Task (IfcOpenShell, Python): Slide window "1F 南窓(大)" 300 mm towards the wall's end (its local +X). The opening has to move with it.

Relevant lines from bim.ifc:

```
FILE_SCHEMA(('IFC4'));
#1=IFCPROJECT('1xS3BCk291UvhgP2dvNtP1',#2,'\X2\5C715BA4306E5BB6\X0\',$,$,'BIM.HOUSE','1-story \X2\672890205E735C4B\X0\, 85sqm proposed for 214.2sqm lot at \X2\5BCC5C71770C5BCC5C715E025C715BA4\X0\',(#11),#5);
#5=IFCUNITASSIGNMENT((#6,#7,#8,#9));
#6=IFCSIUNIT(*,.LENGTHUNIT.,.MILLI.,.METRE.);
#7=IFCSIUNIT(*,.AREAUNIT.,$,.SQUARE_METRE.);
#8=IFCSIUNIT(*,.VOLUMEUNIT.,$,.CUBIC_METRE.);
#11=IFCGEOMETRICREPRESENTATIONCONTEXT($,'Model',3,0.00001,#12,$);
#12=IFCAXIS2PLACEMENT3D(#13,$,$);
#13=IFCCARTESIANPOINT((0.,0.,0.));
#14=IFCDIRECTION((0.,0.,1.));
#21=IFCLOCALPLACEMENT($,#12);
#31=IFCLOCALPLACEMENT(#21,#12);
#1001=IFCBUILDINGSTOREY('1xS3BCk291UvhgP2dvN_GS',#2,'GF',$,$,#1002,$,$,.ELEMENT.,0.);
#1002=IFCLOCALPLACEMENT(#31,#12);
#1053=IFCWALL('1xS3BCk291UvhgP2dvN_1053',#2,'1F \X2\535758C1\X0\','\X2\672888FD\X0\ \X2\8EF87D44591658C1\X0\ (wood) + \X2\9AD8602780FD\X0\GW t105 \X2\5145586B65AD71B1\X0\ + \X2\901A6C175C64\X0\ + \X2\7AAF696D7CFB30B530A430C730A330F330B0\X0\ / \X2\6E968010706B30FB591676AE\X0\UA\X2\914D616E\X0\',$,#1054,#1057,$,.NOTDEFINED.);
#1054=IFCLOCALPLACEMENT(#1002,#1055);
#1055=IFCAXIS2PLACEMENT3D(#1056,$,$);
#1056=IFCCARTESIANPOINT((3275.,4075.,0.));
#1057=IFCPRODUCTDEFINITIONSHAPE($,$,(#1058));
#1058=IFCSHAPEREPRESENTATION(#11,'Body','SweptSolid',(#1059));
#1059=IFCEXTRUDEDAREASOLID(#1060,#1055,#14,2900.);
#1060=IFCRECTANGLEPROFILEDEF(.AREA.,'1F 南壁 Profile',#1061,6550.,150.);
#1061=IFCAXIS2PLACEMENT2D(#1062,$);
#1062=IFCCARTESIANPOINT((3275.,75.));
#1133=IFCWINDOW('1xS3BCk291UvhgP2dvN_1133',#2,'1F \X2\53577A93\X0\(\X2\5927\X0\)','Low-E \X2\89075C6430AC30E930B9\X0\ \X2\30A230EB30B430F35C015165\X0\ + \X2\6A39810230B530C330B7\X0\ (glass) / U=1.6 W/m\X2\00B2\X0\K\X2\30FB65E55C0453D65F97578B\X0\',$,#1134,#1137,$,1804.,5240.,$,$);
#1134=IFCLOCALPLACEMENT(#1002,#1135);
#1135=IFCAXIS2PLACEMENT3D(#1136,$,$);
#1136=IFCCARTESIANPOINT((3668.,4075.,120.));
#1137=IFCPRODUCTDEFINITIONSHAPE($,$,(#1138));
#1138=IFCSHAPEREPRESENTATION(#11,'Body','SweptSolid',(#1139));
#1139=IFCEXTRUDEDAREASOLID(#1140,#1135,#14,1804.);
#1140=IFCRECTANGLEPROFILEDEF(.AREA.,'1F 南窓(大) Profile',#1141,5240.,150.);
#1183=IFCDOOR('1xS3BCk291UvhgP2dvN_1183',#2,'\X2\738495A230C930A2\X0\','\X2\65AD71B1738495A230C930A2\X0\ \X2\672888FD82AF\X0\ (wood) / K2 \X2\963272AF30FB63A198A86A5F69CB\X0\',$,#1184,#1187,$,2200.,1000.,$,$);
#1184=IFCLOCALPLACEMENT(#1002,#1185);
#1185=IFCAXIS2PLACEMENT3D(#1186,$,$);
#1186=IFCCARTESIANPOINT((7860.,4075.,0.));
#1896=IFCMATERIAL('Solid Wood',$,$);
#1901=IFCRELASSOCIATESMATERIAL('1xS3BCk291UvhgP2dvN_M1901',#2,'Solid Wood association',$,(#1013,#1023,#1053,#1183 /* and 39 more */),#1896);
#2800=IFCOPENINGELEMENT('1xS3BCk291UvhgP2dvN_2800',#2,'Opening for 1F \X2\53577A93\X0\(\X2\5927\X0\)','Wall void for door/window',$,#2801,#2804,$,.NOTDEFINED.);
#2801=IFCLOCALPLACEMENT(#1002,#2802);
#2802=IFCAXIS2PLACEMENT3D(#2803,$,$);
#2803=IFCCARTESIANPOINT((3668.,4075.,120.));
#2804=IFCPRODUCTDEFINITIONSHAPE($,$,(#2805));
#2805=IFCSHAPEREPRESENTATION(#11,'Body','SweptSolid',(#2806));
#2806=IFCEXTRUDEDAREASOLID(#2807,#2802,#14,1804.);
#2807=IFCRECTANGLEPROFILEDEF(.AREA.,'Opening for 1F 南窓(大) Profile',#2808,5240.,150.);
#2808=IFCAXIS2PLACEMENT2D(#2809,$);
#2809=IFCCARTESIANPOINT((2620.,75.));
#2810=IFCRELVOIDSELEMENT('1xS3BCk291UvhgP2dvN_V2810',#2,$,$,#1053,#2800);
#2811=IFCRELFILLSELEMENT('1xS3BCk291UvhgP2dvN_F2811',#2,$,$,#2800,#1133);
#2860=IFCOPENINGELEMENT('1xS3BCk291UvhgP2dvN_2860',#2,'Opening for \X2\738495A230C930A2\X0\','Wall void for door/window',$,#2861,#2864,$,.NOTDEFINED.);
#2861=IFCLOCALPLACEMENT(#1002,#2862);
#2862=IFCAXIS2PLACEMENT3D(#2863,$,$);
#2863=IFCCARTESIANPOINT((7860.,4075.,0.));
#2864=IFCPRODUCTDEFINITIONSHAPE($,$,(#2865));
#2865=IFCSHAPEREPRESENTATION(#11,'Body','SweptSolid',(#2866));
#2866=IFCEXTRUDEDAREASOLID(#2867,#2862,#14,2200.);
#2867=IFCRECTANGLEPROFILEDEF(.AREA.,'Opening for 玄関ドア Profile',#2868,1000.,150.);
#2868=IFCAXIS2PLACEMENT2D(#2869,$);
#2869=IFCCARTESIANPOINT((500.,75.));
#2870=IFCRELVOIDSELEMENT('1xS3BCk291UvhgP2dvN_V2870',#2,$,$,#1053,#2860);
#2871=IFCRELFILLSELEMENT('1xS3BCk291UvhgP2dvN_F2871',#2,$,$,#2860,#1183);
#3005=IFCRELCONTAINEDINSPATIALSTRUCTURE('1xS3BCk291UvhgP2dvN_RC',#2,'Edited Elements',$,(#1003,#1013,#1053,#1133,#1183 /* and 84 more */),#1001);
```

```python
import ifcopenshell
import ifcopenshell.api.geometry
import ifcopenshell.util.placement

model = ifcopenshell.open("bim.ifc")

window = model.by_id(1133)
opening = window.FillsVoids[0].RelatingOpeningElement
wall = opening.VoidsElements[0].RelatingBuildingElement

wall_matrix = ifcopenshell.util.placement.get_local_placement(wall.ObjectPlacement)
shift = wall_matrix[:3, 0] * 300.0
before = ifcopenshell.util.placement.get_local_placement(window.ObjectPlacement)[:3, 3].copy()

# The window is not placed relative to its opening, so move both.
for product in (opening, window):
    matrix = ifcopenshell.util.placement.get_local_placement(product.ObjectPlacement)
    matrix[:3, 3] += shift
    ifcopenshell.api.geometry.edit_object_placement(model, product=product, matrix=matrix, is_si=False)

after = ifcopenshell.util.placement.get_local_placement(window.ObjectPlacement)[:3, 3]
print("window moved by", (after - before).round(3) + 0.0)

model.write("bim_edited.ifc")
```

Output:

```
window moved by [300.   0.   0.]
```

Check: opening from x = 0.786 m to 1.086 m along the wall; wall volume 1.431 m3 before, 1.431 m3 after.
